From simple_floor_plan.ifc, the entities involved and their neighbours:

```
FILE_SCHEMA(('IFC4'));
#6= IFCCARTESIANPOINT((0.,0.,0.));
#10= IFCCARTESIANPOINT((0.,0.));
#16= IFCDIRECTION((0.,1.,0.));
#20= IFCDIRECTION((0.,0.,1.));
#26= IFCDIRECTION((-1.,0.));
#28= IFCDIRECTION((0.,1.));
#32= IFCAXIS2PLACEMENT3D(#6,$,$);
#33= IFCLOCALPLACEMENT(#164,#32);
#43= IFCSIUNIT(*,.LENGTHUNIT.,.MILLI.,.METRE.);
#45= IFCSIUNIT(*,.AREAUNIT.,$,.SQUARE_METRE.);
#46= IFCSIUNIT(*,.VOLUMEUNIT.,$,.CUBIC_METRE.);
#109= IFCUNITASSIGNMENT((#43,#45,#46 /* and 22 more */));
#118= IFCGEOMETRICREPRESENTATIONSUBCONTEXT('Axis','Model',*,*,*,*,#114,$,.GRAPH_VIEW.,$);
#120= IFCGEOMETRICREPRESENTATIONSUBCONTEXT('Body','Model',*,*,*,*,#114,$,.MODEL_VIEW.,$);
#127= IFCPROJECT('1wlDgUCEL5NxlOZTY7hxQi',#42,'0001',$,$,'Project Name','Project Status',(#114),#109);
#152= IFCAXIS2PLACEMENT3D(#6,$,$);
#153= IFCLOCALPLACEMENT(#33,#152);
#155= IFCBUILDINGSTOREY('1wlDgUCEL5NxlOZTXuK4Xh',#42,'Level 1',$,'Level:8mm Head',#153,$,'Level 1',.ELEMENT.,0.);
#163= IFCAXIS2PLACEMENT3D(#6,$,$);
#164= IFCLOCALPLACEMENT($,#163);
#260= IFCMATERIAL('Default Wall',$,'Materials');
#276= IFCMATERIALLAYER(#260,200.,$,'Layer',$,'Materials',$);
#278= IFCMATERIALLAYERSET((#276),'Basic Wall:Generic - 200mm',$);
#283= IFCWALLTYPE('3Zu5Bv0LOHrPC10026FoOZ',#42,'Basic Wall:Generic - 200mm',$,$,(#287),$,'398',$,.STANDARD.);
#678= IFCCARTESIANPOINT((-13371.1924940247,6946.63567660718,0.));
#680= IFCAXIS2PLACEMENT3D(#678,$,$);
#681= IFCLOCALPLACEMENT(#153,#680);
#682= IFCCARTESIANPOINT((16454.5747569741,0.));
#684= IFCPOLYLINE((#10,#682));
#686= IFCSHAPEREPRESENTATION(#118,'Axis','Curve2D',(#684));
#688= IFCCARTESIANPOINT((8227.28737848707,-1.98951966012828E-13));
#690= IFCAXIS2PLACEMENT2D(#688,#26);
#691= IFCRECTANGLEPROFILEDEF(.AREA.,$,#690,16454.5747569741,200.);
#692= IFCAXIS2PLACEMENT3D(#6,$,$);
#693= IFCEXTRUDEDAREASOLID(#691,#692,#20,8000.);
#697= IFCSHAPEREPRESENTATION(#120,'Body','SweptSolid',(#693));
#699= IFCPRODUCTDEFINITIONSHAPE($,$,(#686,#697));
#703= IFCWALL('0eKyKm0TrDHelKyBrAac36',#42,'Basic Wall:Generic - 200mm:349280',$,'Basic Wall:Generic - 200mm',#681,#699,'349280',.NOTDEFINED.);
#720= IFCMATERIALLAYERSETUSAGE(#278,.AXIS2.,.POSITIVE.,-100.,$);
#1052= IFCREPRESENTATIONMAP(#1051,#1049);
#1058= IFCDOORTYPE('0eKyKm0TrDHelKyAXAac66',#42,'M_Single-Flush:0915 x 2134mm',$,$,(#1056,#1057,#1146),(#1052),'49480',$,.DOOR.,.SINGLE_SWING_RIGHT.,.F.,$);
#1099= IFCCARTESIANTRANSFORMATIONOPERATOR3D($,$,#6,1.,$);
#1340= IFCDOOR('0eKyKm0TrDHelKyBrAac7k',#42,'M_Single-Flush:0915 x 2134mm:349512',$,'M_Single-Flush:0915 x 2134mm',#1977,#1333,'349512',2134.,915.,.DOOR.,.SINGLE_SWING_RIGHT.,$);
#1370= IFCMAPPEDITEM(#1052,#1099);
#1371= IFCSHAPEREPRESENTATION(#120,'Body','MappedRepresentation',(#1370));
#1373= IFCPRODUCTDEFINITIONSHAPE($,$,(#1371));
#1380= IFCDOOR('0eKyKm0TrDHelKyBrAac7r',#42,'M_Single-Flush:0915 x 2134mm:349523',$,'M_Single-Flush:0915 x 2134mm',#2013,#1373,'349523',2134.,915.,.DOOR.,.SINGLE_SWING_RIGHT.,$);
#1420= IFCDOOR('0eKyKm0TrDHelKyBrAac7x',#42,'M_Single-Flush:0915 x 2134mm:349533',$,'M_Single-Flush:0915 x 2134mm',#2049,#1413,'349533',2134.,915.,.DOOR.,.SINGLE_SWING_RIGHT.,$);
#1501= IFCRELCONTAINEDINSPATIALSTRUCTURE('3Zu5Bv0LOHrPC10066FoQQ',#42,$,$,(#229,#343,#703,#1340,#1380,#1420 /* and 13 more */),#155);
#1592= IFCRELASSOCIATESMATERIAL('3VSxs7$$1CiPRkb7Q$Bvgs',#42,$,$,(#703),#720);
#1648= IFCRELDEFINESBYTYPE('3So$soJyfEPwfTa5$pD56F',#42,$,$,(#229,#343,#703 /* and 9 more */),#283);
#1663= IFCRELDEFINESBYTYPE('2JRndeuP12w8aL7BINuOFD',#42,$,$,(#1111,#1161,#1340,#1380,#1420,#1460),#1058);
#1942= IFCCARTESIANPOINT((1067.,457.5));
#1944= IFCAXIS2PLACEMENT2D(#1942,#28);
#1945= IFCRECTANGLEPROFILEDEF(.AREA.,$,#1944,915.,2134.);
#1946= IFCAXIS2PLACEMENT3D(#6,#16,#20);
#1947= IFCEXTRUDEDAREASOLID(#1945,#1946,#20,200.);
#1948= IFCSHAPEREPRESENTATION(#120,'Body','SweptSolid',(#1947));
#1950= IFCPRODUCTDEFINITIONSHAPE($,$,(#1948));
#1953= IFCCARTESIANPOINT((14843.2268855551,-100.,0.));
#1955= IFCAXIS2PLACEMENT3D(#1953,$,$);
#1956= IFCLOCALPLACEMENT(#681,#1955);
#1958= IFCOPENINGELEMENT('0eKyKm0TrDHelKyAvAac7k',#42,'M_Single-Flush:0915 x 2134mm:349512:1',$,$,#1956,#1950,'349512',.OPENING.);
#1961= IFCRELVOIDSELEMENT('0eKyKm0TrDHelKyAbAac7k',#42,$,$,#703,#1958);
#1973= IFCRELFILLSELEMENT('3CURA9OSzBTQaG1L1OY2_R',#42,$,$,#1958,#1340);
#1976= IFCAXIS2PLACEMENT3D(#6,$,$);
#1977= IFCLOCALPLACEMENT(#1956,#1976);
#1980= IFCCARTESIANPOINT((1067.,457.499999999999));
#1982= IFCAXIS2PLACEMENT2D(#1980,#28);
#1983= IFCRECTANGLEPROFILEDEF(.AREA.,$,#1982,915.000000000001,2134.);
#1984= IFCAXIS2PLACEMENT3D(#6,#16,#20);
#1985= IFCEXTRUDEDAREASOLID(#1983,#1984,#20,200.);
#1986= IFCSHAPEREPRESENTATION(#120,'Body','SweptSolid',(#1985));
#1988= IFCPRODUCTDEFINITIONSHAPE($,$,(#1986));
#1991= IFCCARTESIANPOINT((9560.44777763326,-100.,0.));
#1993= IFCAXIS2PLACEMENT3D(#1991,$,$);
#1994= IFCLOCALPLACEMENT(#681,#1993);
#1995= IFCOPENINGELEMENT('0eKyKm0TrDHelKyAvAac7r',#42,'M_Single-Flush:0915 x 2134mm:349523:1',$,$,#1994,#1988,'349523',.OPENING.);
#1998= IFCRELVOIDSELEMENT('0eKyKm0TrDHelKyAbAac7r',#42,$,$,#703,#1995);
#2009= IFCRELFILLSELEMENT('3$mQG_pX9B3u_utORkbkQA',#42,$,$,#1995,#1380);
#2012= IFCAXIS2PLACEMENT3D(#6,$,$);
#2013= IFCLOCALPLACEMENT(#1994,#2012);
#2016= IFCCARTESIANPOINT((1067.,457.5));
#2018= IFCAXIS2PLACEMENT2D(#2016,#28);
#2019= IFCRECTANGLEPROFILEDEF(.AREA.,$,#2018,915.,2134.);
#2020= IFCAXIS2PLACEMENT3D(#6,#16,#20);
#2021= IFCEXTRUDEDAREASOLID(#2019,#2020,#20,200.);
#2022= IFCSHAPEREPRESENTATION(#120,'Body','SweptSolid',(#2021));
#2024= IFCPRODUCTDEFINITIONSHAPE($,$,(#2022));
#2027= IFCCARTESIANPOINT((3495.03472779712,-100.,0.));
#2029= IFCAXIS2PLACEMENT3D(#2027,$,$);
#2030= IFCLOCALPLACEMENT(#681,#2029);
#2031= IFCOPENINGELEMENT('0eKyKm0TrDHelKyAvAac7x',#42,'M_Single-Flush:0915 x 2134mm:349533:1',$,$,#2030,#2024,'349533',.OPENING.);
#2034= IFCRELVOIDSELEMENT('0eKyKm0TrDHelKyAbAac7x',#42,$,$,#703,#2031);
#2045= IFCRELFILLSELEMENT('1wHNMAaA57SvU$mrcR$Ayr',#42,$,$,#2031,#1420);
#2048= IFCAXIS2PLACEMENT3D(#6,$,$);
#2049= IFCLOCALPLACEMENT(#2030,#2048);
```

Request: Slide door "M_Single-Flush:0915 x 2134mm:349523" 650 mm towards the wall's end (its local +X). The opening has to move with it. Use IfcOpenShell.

```python
import ifcopenshell
import ifcopenshell.api.geometry
import ifcopenshell.util.placement

model = ifcopenshell.open("simple_floor_plan.ifc")

door = model.by_id(1380)
opening = door.FillsVoids[0].RelatingOpeningElement
wall = opening.VoidsElements[0].RelatingBuildingElement

wall_matrix = ifcopenshell.util.placement.get_local_placement(wall.ObjectPlacement)
shift = wall_matrix[:3, 0] * 650.0
before = ifcopenshell.util.placement.get_local_placement(door.ObjectPlacement)[:3, 3].copy()

# The door is placed relative to its opening, so it follows when the opening moves.
matrix = ifcopenshell.util.placement.get_local_placement(opening.ObjectPlacement)
matrix[:3, 3] += shift
ifcopenshell.api.geometry.edit_object_placement(
    model, product=opening, matrix=matrix, is_si=False, should_transform_children=True
)

after = ifcopenshell.util.placement.get_local_placement(door.ObjectPlacement)[:3, 3]
print("door moved by", (after - before).round(3) + 0.0)

model.write("simple_floor_plan_edited.ifc")
```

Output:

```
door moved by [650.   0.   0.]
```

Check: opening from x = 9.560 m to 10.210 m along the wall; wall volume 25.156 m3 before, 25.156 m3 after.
